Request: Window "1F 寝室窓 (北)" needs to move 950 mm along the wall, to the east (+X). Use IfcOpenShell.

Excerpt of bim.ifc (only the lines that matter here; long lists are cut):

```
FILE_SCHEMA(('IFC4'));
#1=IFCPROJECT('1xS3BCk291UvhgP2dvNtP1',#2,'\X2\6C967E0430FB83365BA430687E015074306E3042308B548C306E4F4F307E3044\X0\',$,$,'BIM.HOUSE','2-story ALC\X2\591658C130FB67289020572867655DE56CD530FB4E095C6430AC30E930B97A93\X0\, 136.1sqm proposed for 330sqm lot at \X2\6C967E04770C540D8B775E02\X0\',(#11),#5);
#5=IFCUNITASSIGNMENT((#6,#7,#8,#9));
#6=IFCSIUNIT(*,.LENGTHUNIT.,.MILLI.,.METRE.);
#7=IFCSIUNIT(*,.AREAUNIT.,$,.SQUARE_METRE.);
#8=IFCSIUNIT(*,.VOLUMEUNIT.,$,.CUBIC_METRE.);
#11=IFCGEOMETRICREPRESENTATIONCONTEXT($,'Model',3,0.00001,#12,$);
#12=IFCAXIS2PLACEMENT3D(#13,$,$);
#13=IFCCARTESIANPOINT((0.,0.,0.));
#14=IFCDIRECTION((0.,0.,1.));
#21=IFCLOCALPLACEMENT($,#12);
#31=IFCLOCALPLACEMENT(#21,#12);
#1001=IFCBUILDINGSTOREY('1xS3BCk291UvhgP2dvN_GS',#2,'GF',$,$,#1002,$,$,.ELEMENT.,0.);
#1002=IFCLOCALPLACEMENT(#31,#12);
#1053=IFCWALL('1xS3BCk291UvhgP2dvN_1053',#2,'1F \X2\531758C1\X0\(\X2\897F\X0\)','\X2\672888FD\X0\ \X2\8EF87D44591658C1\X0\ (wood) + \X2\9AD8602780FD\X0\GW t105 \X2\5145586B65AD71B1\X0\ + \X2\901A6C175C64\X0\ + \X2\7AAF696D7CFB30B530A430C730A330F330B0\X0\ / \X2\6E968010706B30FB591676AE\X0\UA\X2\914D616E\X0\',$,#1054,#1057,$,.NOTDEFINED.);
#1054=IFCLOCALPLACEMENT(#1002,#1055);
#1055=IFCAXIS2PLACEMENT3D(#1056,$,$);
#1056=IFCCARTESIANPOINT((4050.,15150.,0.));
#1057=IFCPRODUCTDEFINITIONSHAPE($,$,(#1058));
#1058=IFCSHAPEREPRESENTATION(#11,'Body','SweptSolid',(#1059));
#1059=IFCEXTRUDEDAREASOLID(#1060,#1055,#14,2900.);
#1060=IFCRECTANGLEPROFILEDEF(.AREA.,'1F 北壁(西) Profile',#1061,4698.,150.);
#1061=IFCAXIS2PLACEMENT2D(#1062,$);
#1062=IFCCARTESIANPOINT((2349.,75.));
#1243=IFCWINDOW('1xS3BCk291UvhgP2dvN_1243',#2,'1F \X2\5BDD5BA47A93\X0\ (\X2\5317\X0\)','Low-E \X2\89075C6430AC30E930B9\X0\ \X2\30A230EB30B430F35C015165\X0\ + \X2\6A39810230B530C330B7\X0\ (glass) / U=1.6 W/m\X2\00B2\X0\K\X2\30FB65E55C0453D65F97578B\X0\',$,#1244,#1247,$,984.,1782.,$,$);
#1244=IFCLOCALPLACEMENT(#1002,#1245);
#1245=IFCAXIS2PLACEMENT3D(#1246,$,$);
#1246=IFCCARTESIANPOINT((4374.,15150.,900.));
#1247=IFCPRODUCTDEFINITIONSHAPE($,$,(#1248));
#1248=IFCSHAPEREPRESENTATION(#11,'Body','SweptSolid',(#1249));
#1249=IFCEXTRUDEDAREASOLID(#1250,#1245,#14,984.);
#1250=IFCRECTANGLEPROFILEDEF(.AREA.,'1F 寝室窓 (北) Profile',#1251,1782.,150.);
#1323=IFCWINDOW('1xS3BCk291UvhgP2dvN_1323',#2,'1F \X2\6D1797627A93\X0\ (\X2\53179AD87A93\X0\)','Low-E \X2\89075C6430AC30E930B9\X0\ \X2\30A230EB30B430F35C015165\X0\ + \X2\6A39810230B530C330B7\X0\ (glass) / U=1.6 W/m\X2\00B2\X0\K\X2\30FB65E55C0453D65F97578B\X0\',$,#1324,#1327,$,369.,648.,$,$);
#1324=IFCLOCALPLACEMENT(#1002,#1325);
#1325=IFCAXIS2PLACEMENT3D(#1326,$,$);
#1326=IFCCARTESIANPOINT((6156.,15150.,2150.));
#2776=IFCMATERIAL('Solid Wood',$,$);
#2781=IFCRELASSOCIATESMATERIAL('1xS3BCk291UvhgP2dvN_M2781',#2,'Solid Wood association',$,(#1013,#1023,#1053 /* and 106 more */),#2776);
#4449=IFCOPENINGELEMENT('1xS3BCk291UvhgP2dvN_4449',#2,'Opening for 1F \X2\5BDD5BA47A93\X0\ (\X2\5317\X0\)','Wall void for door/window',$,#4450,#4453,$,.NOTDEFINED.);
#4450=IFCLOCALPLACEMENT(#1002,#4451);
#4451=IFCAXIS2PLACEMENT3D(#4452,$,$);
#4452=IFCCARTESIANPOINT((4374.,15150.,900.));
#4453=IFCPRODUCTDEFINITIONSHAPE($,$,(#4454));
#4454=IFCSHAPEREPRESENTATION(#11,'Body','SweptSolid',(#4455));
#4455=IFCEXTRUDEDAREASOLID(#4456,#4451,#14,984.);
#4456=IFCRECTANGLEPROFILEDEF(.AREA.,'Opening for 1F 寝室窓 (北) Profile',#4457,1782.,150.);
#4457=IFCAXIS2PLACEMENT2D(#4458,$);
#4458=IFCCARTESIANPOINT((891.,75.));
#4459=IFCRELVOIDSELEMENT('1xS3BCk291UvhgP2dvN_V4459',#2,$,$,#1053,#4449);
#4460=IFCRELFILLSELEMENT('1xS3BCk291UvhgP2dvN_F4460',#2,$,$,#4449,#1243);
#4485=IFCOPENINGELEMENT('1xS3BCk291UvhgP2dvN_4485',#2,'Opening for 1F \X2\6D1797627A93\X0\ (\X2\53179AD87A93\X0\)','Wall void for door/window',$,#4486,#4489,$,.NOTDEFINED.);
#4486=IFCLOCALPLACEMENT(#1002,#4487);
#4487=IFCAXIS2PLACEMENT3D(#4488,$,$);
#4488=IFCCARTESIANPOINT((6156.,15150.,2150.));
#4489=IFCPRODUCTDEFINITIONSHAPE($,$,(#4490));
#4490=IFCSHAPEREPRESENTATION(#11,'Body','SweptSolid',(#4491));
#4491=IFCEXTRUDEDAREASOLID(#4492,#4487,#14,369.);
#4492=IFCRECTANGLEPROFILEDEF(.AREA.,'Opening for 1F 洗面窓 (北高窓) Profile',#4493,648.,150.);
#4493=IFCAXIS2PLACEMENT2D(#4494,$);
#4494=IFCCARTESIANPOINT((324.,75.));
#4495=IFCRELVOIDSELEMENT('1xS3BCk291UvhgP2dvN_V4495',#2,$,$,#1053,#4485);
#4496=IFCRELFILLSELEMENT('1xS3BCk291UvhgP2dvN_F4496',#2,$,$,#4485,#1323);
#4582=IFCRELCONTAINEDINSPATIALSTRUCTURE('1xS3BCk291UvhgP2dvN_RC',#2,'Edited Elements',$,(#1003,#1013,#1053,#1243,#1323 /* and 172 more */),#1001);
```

```python
import ifcopenshell
import ifcopenshell.api.geometry
import ifcopenshell.util.placement
import ifcopenshell.util.unit

model = ifcopenshell.open("bim.ifc")
unit_scale = ifcopenshell.util.unit.calculate_unit_scale(model)

window = model.by_guid("1xS3BCk291UvhgP2dvN_1243")
opening = window.FillsVoids[0].RelatingOpeningElement
wall = opening.VoidsElements[0].RelatingBuildingElement

wall_matrix = ifcopenshell.util.placement.get_local_placement(wall.ObjectPlacement)
shift = wall_matrix[:3, 0] * 0.95 / unit_scale
before = ifcopenshell.util.placement.get_local_placement(window.ObjectPlacement)[:3, 3].copy()

# The window is not placed relative to its opening, so move both.
for product in (opening, window):
    matrix = ifcopenshell.util.placement.get_local_placement(product.ObjectPlacement)
    matrix[:3, 3] += shift
    ifcopenshell.api.geometry.edit_object_placement(model, product=product, matrix=matrix, is_si=False)

after = ifcopenshell.util.placement.get_local_placement(window.ObjectPlacement)[:3, 3]
print("window moved by", (after - before).round(3) + 0.0)

model.write("bim-out.ifc")
```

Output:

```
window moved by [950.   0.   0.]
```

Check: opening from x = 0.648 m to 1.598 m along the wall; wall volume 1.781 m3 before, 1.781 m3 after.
